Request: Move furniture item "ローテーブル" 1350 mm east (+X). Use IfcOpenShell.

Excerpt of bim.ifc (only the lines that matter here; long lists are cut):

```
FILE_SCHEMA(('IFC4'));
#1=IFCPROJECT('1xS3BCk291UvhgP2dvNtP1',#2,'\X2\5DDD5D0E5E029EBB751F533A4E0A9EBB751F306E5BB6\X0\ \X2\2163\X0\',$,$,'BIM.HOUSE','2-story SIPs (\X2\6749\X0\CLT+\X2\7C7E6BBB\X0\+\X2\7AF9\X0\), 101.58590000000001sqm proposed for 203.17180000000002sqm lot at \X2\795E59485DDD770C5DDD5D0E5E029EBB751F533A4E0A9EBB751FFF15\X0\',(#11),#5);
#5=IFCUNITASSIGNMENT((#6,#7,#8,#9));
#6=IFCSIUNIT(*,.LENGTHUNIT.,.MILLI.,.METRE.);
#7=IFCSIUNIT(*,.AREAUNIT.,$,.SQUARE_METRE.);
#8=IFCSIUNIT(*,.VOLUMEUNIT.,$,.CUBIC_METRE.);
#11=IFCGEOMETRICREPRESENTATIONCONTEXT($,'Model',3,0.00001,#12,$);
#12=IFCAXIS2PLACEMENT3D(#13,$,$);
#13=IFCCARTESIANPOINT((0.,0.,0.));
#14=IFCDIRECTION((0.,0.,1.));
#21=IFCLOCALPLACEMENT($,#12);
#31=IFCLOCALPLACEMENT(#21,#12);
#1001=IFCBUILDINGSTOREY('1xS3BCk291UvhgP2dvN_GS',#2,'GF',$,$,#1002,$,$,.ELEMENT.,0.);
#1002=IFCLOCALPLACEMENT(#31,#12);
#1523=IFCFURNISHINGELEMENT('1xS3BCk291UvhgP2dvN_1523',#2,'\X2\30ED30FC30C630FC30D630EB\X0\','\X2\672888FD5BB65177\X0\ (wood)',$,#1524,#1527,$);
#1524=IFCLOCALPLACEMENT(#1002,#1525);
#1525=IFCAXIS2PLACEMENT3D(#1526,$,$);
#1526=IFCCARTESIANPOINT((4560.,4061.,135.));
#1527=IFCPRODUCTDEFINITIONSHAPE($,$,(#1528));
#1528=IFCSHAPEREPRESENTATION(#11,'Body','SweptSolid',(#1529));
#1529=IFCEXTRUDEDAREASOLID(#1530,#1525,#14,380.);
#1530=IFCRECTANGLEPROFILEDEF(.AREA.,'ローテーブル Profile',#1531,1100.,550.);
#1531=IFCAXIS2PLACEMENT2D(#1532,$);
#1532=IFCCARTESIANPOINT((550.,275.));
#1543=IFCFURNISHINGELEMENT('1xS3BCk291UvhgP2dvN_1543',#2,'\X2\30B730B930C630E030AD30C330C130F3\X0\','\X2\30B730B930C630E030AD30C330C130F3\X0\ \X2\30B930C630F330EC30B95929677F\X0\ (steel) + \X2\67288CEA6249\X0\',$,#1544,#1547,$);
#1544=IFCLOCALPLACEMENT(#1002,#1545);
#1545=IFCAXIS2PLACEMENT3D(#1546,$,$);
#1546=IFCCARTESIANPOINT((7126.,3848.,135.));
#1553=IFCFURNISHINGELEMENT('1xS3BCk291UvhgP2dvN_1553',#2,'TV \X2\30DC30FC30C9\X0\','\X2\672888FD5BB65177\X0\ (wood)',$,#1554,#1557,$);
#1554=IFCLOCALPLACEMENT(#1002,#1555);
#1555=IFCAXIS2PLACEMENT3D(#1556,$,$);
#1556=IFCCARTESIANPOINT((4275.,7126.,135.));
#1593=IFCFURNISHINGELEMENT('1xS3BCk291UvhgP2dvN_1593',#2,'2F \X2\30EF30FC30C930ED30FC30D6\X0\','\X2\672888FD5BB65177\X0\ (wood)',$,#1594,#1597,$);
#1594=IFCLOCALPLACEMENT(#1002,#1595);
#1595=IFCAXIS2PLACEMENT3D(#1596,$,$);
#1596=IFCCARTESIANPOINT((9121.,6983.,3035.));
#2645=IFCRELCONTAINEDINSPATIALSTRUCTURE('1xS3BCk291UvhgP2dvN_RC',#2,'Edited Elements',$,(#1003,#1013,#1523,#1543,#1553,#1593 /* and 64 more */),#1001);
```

```python
import ifcopenshell
import ifcopenshell.api.geometry
import ifcopenshell.util.placement

model = ifcopenshell.open("bim.ifc")

item = model.by_id(1523)
matrix = ifcopenshell.util.placement.get_local_placement(item.ObjectPlacement)
matrix[0, 3] += 1350.0
ifcopenshell.api.geometry.edit_object_placement(model, product=item, matrix=matrix, is_si=False)

print(ifcopenshell.util.placement.get_local_placement(item.ObjectPlacement).round(3) + 0.0)

model.write("bim_edited.ifc")
```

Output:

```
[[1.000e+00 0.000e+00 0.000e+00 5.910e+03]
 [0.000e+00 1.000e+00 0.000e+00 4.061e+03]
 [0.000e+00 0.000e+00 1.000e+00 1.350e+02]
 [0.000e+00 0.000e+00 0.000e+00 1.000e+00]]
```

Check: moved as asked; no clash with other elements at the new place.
